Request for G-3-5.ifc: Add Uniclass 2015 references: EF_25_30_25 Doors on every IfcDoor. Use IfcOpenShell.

First a look at what the model holds.

```python
import ifcopenshell

model = ifcopenshell.open("G-3-5.ifc")
print(model.schema)
print("classifications:", [c.Name for c in model.by_type("IfcClassification")])
for ifc_class in ("IfcDoor", "IfcRoof", "IfcStair", "IfcWall", "IfcWindow"):
    print(ifc_class, len(model.by_type(ifc_class)))
```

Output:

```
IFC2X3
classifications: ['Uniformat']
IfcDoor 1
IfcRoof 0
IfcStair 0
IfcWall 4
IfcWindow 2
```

```python
import ifcopenshell
import ifcopenshell.api.classification

model = ifcopenshell.open("G-3-5.ifc")

# IFC2X3 requires Source and Edition and has no link from the project to the system.
system = model.create_entity("IfcClassification", Source="NBS", Edition="2015", Name="Uniclass 2015")

codes = {
    "IfcDoor": ("EF_25_30_25", "Doors"),
}
for ifc_class, (code, name) in codes.items():
    products = model.by_type(ifc_class)
    ifcopenshell.api.classification.add_reference(
        model, products=products, classification=system, identification=code, name=name
    )
    print(code, len(products))

model.write("G-3-5-out.ifc")
```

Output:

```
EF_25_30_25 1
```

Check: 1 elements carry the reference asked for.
